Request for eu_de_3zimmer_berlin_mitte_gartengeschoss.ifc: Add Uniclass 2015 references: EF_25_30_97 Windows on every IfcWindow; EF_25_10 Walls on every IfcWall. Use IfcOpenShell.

First a look at what the model holds.

```python
import ifcopenshell

model = ifcopenshell.open("eu_de_3zimmer_berlin_mitte_gartengeschoss.ifc")
print(model.schema)
print("classifications:", [c.Name for c in model.by_type("IfcClassification")])
for ifc_class in ("IfcDoor", "IfcRoof", "IfcStair", "IfcWall", "IfcWindow"):
    print(ifc_class, len(model.by_type(ifc_class)))
```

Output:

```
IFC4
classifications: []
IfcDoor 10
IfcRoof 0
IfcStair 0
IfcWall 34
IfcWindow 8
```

```python
import ifcopenshell
import ifcopenshell.api.classification

model = ifcopenshell.open("eu_de_3zimmer_berlin_mitte_gartengeschoss.ifc")

system = ifcopenshell.api.classification.add_classification(model, classification="Uniclass 2015")

codes = {
    "IfcWindow": ("EF_25_30_97", "Windows"),
    "IfcWall": ("EF_25_10", "Walls"),
}
for ifc_class, (code, name) in codes.items():
    products = model.by_type(ifc_class)
    ifcopenshell.api.classification.add_reference(
        model, products=products, classification=system, identification=code, name=name
    )
    print(code, len(products))

model.write("eu_de_3zimmer_berlin_mitte_gartengeschoss_rev.ifc")
```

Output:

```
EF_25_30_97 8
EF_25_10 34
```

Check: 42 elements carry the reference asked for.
